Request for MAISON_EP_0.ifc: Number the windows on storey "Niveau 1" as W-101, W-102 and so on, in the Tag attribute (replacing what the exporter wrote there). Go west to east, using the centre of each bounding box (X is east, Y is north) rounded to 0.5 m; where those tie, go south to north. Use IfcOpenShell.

First a look at what the model holds.

```python
import ifcopenshell
import ifcopenshell.util.element
import ifcopenshell.util.placement

model = ifcopenshell.open("MAISON_EP_0.ifc")
print(model.schema)
storey = next(s for s in model.by_type("IfcBuildingStorey") if s.Name == "Niveau 1")
windows = [e for e in ifcopenshell.util.element.get_decomposition(storey) if e.is_a("IfcWindow")]
for e in sorted(windows, key=lambda e: e.id()):
    origin = ifcopenshell.util.placement.get_local_placement(e.ObjectPlacement)[:3, 3]
    print(e.id(), e.Tag, e.Name, origin.round(2) + 0.0, sep=" | ")
```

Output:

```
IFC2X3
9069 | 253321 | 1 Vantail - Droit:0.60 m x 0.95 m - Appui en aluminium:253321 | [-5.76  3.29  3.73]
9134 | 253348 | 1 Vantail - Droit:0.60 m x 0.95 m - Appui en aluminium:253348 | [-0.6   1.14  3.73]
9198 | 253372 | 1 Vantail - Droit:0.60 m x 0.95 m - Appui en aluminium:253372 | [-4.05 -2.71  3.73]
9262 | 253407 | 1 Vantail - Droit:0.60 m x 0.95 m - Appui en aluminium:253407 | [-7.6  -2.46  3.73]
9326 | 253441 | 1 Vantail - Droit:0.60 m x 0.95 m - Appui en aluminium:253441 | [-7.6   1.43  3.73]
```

```python
import ifcopenshell
import ifcopenshell.geom
import ifcopenshell.util.element
import ifcopenshell.util.shape

model = ifcopenshell.open("MAISON_EP_0.ifc")
settings = ifcopenshell.geom.settings()
settings.set("use-world-coords", True)


def centre(element):
    shape = ifcopenshell.geom.create_shape(settings, element)
    return ifcopenshell.util.shape.get_bbox_centroid(shape.geometry)


storey = next(s for s in model.by_type("IfcBuildingStorey") if s.Name == "Niveau 1")
windows = [e for e in ifcopenshell.util.element.get_decomposition(storey) if e.is_a("IfcWindow")]

# Insertion points can sit at a corner or the storey origin, so sort by the geometry (in metres).
centres = {e: centre(e) for e in windows}
windows.sort(key=lambda e: (round(centres[e][0] / 0.5), centres[e][1]))

for i, e in enumerate(windows, start=1):
    number = f"W-1{i:02d}"
    e.Tag = number
    print(e.id(), number)

model.write("MAISON_EP_0_rev.ifc")
```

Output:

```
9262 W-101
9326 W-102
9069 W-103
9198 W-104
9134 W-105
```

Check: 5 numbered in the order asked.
